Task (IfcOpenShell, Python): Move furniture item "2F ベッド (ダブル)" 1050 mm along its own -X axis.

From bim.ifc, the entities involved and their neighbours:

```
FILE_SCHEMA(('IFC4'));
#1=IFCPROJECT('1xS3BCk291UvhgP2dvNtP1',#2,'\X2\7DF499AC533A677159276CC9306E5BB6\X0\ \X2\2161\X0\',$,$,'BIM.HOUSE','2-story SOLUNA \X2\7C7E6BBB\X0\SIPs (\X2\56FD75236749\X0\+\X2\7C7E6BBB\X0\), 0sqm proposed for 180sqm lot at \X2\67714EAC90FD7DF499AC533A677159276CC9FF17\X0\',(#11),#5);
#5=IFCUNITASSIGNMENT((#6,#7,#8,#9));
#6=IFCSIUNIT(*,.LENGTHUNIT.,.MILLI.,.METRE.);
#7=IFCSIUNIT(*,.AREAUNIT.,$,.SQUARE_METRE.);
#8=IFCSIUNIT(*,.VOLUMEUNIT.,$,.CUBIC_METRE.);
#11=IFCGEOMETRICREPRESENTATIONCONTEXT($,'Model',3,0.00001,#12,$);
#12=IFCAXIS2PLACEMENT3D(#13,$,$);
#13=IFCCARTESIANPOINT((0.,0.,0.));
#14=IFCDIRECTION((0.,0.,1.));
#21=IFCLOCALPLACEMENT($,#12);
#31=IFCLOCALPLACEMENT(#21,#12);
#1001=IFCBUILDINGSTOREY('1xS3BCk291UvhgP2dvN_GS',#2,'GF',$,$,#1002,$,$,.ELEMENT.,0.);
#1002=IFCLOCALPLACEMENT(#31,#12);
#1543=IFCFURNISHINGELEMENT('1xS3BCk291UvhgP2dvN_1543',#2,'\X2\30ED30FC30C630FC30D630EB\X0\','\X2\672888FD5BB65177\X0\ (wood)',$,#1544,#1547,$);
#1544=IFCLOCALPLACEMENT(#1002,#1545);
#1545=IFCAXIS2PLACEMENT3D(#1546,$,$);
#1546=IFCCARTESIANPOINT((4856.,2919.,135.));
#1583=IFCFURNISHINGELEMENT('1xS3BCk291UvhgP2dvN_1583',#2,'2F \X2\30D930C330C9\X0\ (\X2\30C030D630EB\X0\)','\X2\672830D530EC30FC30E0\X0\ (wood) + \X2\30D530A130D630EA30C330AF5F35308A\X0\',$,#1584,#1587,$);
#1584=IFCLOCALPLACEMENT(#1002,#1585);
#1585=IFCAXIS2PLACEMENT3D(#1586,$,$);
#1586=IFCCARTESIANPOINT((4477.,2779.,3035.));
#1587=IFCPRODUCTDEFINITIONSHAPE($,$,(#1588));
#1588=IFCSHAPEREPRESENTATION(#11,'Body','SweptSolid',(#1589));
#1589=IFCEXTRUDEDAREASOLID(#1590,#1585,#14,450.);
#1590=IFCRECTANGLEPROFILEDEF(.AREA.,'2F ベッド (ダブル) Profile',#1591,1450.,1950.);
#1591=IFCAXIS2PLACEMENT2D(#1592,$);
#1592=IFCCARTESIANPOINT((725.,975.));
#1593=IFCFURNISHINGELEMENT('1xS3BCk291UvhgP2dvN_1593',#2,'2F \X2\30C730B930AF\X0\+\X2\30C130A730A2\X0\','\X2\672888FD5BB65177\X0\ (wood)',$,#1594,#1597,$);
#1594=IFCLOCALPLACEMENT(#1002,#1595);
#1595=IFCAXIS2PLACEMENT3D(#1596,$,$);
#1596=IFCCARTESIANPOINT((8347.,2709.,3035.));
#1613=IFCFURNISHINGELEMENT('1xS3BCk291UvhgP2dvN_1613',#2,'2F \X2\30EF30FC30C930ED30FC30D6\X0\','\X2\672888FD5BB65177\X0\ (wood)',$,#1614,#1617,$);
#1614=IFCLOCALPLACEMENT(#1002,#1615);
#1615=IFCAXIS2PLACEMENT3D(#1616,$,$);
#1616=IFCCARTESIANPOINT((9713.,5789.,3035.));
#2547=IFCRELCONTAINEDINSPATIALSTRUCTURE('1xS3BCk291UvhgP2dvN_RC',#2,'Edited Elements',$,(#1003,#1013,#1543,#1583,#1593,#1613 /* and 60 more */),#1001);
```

```python
import ifcopenshell
import ifcopenshell.api.geometry
import ifcopenshell.util.placement
import ifcopenshell.util.unit

model = ifcopenshell.open("bim.ifc")
unit_scale = ifcopenshell.util.unit.calculate_unit_scale(model)

item = model.by_guid("1xS3BCk291UvhgP2dvN_1583")
matrix = ifcopenshell.util.placement.get_local_placement(item.ObjectPlacement)
matrix[:3, 3] -= matrix[:3, 0] * 1.05 / unit_scale
ifcopenshell.api.geometry.edit_object_placement(model, product=item, matrix=matrix, is_si=False)

print(ifcopenshell.util.placement.get_local_placement(item.ObjectPlacement).round(3) + 0.0)

model.write("bim_edited.ifc")
```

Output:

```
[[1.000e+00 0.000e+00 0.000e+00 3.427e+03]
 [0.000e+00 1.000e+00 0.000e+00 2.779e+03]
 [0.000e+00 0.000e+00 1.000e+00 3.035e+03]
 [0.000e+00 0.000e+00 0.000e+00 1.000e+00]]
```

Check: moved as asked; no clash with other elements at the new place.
